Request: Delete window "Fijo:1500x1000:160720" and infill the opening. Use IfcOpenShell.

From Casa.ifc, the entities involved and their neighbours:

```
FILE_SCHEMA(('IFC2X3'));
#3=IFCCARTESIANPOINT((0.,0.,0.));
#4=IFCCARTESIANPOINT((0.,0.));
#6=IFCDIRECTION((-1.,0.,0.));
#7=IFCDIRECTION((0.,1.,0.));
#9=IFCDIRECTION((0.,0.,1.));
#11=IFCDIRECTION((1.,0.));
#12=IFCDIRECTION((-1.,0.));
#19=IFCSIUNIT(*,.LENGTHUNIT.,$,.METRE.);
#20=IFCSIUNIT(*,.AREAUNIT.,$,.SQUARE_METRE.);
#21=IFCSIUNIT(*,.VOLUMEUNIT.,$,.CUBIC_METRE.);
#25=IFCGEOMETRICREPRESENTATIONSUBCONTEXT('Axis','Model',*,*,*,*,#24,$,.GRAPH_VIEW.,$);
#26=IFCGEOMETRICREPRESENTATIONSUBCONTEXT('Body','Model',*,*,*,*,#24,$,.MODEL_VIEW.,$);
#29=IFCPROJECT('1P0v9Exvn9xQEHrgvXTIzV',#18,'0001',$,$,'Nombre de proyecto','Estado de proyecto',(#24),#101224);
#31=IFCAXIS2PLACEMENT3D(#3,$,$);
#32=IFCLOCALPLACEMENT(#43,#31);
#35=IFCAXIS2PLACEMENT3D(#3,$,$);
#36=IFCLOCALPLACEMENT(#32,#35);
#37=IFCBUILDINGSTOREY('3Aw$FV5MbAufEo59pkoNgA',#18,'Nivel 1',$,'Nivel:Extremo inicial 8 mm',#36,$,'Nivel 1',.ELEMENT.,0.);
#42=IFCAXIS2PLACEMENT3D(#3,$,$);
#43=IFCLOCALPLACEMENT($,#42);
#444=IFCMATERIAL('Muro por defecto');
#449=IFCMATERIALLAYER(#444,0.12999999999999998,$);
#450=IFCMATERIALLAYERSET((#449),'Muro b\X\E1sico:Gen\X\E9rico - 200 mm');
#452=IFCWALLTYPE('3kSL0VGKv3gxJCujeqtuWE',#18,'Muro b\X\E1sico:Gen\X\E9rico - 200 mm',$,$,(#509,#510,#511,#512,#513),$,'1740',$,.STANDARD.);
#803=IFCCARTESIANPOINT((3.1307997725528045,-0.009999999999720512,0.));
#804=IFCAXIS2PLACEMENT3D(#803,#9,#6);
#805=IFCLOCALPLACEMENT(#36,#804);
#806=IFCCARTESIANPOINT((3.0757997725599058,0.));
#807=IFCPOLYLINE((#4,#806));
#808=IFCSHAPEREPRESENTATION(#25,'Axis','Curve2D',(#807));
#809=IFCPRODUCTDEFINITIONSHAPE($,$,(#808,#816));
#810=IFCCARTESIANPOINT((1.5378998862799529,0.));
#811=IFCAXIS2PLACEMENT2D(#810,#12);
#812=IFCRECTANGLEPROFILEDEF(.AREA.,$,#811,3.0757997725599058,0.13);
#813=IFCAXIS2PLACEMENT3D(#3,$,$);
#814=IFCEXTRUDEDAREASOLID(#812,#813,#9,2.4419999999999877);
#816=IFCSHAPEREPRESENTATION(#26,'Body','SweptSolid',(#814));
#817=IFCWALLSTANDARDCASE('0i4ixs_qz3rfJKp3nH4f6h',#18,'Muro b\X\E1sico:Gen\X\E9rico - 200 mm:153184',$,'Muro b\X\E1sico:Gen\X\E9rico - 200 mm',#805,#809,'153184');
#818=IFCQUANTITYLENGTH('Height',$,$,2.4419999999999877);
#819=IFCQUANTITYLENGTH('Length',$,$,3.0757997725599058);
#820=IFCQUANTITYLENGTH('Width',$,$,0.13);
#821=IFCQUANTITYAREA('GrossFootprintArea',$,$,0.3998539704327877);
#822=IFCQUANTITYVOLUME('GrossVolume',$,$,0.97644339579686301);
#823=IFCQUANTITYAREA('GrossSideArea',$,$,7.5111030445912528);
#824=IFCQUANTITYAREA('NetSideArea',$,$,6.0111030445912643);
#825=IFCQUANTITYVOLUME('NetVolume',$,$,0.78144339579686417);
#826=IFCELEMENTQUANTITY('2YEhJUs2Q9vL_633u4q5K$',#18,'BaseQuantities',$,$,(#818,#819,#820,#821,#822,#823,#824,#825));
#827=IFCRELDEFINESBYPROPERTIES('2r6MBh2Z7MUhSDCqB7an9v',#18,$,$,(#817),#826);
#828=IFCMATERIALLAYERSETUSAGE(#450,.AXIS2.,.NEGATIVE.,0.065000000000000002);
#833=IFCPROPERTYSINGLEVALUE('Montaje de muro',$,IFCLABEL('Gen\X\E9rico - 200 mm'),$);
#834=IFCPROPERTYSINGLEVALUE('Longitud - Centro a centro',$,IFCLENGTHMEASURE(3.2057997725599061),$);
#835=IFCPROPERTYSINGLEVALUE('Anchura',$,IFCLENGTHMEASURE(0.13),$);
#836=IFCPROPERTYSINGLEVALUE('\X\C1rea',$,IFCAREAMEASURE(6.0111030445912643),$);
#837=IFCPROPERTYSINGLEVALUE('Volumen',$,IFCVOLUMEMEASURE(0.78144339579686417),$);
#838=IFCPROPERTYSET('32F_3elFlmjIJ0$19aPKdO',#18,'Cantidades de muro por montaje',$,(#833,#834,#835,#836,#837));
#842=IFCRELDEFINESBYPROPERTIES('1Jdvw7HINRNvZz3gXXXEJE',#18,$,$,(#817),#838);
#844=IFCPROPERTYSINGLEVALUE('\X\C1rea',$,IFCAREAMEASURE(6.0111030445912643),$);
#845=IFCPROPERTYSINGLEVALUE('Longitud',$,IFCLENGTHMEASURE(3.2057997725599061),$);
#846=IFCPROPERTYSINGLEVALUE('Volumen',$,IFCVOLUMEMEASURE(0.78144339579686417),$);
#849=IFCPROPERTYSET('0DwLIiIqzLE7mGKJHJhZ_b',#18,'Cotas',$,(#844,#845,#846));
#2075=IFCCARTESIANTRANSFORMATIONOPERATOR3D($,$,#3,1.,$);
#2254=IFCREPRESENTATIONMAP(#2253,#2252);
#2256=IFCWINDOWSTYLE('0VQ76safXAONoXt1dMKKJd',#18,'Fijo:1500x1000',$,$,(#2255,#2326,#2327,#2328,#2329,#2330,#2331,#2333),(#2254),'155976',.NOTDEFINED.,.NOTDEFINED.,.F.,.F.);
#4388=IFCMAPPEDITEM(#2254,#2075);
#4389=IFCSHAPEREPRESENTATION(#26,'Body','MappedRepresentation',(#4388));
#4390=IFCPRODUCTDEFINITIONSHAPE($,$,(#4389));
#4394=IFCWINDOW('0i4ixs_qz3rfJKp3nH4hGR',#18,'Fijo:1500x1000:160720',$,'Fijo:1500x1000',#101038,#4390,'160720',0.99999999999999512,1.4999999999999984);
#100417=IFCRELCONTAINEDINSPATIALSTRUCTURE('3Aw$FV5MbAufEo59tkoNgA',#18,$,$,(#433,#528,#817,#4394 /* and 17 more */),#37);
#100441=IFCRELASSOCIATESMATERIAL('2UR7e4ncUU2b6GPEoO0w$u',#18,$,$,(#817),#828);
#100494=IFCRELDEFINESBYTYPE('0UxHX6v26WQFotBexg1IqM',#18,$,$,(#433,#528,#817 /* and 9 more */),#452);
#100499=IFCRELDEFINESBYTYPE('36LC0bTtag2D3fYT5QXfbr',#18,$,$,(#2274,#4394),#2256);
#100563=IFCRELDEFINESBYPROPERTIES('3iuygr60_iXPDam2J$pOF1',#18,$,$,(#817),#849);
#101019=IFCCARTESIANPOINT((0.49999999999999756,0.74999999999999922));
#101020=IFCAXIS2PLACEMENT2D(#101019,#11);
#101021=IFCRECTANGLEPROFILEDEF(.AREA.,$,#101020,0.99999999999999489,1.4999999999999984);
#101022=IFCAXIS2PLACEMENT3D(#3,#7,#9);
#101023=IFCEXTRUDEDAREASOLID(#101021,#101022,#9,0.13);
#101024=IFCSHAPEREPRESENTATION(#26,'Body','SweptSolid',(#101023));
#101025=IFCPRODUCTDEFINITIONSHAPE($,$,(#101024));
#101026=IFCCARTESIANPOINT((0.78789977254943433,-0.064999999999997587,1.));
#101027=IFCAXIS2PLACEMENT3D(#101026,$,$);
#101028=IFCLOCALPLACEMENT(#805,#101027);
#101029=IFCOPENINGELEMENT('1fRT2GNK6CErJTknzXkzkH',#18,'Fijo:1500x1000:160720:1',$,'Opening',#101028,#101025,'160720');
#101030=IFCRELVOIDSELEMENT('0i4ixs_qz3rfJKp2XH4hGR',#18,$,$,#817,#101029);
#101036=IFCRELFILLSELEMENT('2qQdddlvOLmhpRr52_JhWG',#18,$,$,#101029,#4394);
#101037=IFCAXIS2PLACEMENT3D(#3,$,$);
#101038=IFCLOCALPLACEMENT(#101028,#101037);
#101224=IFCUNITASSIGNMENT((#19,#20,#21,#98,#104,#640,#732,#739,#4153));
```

```python
import ifcopenshell
import ifcopenshell.api.feature
import ifcopenshell.api.pset
import ifcopenshell.api.root
import ifcopenshell.geom
import ifcopenshell.util.element
import ifcopenshell.util.shape
import ifcopenshell.util.unit

model = ifcopenshell.open("Casa.ifc")
area_scale = ifcopenshell.util.unit.calculate_unit_scale(model, "AREAUNIT")
volume_scale = ifcopenshell.util.unit.calculate_unit_scale(model, "VOLUMEUNIT")
settings = ifcopenshell.geom.settings()


def volume(element):
    """Net volume in cubic metres, openings subtracted."""
    shape = ifcopenshell.geom.create_shape(settings, element)
    return ifcopenshell.util.shape.get_volume(shape.geometry)


window = model.by_guid("0i4ixs_qz3rfJKp3nH4hGR")
opening = window.FillsVoids[0].RelatingOpeningElement
wall = opening.VoidsElements[0].RelatingBuildingElement
before = volume(wall)

ifcopenshell.api.root.remove_product(model, product=window)
ifcopenshell.api.feature.remove_feature(model, feature=opening)

after = volume(wall)
thickness = 0.13  # wall thickness in metres

# Update the wall's stored quantities.
qto = model.by_id(ifcopenshell.util.element.get_pset(wall, "BaseQuantities", should_inherit=False)["id"])
ifcopenshell.api.pset.edit_qto(model, qto=qto, properties={
    "NetSideArea": after / thickness / area_scale,
    "NetVolume": after / volume_scale,
})
pset = model.by_id(ifcopenshell.util.element.get_pset(wall, "Cantidades de muro por montaje", should_inherit=False)["id"])
ifcopenshell.api.pset.edit_pset(model, pset=pset, properties={
    "Área": model.create_entity("IfcAreaMeasure", after / thickness / area_scale),
    "Volumen": model.create_entity("IfcVolumeMeasure", after / volume_scale),
})
pset = model.by_id(ifcopenshell.util.element.get_pset(wall, "Cotas", should_inherit=False)["id"])
ifcopenshell.api.pset.edit_pset(model, pset=pset, properties={
    "Área": model.create_entity("IfcAreaMeasure", after / thickness / area_scale),
    "Volumen": model.create_entity("IfcVolumeMeasure", after / volume_scale),
})

print(f"wall volume {before:.3f} -> {after:.3f} m3")

model.write("Casa_edited.ifc")
```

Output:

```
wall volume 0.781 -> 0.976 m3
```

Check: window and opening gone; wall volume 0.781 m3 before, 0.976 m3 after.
